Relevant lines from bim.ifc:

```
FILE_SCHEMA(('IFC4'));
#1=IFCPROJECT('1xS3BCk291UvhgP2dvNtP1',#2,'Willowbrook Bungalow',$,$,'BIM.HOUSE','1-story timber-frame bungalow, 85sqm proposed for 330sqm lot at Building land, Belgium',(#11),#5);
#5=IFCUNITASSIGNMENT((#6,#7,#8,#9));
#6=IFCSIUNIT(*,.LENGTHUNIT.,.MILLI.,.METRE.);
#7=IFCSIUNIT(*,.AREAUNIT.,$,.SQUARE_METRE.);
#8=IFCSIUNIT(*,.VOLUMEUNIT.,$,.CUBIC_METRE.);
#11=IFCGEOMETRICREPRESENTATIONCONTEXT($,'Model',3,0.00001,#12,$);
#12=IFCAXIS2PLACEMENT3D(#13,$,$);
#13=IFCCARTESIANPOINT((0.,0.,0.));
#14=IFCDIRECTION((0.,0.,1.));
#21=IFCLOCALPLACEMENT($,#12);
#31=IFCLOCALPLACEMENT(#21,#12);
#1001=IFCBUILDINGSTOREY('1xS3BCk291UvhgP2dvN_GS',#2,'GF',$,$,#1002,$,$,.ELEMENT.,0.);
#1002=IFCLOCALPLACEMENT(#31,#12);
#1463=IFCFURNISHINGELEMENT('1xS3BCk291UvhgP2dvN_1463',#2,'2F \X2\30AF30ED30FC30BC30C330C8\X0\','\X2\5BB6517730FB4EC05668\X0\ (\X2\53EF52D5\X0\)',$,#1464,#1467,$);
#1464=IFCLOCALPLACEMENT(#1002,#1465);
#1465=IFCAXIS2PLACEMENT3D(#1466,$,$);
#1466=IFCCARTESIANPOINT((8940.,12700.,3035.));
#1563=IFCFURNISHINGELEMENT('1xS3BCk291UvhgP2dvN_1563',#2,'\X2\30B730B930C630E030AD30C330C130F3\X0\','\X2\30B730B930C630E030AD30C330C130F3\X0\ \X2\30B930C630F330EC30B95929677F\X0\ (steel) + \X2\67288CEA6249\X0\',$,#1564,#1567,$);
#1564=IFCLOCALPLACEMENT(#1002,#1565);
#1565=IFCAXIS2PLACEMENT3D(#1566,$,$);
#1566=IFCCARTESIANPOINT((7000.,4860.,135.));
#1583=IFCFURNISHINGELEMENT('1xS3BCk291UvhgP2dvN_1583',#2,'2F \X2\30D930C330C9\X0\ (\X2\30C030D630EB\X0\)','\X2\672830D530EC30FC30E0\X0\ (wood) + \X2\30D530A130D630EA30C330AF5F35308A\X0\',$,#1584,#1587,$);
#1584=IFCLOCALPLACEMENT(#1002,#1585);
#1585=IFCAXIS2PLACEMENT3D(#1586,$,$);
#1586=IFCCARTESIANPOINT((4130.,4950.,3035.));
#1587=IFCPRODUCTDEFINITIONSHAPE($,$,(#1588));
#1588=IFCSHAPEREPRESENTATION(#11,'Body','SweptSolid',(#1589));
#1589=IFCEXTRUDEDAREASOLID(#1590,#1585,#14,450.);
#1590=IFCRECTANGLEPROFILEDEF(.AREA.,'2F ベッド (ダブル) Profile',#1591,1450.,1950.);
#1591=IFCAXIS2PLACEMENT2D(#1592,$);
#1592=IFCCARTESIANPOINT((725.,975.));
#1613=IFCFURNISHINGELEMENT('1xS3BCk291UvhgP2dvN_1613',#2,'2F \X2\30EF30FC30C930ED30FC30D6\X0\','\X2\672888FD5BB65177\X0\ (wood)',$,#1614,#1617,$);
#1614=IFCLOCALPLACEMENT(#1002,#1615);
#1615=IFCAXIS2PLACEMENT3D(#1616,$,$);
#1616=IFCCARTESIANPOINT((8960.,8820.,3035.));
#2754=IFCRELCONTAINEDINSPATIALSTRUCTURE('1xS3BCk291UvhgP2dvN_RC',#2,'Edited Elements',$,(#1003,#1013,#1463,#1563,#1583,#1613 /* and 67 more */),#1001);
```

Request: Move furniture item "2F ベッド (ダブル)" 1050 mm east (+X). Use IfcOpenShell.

```python
import ifcopenshell
import ifcopenshell.api.geometry
import ifcopenshell.util.placement

model = ifcopenshell.open("bim.ifc")

item = model.by_id(1583)
matrix = ifcopenshell.util.placement.get_local_placement(item.ObjectPlacement)
matrix[0, 3] += 1050.0
ifcopenshell.api.geometry.edit_object_placement(model, product=item, matrix=matrix, is_si=False)

print(ifcopenshell.util.placement.get_local_placement(item.ObjectPlacement).round(3) + 0.0)

model.write("bim-out.ifc")
```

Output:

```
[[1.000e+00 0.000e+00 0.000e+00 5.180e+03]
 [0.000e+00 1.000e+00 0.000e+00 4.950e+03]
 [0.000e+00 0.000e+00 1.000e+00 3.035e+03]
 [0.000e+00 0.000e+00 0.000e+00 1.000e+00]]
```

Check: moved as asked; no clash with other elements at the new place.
